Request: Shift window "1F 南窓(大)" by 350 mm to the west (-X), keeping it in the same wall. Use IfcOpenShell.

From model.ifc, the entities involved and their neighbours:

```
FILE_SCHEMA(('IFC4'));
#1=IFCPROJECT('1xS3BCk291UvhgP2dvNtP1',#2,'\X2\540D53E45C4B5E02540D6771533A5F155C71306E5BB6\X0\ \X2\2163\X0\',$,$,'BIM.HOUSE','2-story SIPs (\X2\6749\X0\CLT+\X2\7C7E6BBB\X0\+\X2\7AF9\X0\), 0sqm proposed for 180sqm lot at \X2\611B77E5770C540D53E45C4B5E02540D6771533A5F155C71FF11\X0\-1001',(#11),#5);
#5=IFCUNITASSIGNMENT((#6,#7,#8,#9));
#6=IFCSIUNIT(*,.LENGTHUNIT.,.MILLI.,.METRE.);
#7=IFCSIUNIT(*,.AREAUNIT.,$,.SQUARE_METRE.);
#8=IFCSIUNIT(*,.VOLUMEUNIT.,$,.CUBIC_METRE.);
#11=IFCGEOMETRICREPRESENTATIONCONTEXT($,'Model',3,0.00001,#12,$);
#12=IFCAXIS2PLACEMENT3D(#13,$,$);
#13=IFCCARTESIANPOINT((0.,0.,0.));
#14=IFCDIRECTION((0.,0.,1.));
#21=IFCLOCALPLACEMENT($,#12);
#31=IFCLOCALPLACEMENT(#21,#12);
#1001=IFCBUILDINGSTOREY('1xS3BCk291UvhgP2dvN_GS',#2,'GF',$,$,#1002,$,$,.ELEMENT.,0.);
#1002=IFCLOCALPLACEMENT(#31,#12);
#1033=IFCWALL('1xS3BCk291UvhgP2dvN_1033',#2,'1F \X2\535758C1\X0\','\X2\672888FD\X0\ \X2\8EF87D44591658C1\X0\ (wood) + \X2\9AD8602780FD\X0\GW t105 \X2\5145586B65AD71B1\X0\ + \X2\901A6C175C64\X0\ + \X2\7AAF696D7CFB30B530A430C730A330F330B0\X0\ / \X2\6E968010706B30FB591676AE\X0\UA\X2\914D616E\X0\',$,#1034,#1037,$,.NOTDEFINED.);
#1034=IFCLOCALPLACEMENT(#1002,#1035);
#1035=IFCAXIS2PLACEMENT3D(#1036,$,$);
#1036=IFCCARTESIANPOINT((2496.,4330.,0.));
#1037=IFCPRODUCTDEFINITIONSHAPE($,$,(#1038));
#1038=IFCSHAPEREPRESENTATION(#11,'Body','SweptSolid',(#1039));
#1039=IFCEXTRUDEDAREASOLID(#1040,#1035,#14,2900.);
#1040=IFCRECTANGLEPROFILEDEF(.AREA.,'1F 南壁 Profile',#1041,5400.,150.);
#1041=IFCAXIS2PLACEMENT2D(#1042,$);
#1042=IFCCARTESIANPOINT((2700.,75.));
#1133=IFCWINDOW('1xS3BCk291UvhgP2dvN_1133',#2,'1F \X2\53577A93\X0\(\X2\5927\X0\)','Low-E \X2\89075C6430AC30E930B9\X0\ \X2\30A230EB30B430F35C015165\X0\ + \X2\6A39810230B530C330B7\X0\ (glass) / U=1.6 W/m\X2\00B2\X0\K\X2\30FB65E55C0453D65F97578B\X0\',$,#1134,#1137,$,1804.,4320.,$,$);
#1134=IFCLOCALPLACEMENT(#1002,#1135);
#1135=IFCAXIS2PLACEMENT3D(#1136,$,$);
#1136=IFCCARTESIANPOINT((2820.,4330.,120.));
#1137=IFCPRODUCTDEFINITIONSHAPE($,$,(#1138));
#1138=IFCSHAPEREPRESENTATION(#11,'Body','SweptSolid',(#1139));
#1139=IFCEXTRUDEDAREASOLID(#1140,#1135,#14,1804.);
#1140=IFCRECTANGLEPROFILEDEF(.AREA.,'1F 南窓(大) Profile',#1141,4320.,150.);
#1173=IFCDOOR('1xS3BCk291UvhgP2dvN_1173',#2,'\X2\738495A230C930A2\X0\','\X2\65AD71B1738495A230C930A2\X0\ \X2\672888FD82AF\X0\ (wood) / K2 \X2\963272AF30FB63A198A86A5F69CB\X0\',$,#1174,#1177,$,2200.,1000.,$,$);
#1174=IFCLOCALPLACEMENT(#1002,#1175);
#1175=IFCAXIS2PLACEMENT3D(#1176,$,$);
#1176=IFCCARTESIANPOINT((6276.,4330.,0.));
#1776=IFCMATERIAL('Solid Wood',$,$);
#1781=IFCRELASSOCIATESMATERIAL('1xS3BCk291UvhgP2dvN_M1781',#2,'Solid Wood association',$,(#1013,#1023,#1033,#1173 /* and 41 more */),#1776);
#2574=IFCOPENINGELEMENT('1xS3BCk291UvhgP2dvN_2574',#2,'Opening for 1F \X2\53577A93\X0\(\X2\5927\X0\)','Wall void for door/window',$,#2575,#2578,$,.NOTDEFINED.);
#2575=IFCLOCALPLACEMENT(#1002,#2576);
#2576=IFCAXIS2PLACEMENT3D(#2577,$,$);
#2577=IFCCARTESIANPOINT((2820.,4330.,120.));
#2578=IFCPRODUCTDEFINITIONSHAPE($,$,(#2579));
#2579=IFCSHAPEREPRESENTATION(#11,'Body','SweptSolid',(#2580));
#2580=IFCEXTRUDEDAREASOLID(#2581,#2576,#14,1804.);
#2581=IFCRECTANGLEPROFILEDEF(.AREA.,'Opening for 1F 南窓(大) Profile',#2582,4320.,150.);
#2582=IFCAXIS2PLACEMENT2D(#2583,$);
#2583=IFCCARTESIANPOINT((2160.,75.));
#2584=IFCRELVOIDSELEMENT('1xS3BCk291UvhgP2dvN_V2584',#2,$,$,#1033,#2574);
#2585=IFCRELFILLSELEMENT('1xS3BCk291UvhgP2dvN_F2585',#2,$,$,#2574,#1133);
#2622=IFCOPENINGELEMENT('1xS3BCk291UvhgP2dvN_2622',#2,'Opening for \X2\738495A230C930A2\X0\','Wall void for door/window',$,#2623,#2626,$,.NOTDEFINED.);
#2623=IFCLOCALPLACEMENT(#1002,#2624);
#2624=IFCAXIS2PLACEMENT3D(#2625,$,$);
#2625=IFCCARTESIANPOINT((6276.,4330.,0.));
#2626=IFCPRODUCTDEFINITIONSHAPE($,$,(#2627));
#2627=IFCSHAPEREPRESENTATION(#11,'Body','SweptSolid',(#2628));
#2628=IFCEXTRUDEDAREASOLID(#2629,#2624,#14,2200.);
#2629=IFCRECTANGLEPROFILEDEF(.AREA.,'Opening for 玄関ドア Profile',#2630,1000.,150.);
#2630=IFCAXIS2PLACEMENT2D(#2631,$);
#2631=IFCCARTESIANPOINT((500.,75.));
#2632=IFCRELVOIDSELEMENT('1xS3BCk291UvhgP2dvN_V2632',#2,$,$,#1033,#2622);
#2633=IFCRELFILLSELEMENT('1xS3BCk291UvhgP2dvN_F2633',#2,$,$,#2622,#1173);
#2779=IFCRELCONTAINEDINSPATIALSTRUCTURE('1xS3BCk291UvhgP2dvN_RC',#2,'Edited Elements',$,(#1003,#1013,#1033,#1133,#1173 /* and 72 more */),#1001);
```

```python
import ifcopenshell
import ifcopenshell.api.geometry
import ifcopenshell.util.placement
import ifcopenshell.util.unit

model = ifcopenshell.open("model.ifc")
unit_scale = ifcopenshell.util.unit.calculate_unit_scale(model)

window = model.by_guid("1xS3BCk291UvhgP2dvN_1133")
opening = window.FillsVoids[0].RelatingOpeningElement
wall = opening.VoidsElements[0].RelatingBuildingElement

wall_matrix = ifcopenshell.util.placement.get_local_placement(wall.ObjectPlacement)
shift = wall_matrix[:3, 0] * -0.35 / unit_scale
before = ifcopenshell.util.placement.get_local_placement(window.ObjectPlacement)[:3, 3].copy()

# The window is not placed relative to its opening, so move both.
for product in (opening, window):
    matrix = ifcopenshell.util.placement.get_local_placement(product.ObjectPlacement)
    matrix[:3, 3] += shift
    ifcopenshell.api.geometry.edit_object_placement(model, product=product, matrix=matrix, is_si=False)

after = ifcopenshell.util.placement.get_local_placement(window.ObjectPlacement)[:3, 3]
print("window moved by", (after - before).round(3) + 0.0)

model.write("model_edited.ifc")
```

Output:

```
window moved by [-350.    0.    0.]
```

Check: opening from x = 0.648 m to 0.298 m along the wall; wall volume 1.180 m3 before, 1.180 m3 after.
